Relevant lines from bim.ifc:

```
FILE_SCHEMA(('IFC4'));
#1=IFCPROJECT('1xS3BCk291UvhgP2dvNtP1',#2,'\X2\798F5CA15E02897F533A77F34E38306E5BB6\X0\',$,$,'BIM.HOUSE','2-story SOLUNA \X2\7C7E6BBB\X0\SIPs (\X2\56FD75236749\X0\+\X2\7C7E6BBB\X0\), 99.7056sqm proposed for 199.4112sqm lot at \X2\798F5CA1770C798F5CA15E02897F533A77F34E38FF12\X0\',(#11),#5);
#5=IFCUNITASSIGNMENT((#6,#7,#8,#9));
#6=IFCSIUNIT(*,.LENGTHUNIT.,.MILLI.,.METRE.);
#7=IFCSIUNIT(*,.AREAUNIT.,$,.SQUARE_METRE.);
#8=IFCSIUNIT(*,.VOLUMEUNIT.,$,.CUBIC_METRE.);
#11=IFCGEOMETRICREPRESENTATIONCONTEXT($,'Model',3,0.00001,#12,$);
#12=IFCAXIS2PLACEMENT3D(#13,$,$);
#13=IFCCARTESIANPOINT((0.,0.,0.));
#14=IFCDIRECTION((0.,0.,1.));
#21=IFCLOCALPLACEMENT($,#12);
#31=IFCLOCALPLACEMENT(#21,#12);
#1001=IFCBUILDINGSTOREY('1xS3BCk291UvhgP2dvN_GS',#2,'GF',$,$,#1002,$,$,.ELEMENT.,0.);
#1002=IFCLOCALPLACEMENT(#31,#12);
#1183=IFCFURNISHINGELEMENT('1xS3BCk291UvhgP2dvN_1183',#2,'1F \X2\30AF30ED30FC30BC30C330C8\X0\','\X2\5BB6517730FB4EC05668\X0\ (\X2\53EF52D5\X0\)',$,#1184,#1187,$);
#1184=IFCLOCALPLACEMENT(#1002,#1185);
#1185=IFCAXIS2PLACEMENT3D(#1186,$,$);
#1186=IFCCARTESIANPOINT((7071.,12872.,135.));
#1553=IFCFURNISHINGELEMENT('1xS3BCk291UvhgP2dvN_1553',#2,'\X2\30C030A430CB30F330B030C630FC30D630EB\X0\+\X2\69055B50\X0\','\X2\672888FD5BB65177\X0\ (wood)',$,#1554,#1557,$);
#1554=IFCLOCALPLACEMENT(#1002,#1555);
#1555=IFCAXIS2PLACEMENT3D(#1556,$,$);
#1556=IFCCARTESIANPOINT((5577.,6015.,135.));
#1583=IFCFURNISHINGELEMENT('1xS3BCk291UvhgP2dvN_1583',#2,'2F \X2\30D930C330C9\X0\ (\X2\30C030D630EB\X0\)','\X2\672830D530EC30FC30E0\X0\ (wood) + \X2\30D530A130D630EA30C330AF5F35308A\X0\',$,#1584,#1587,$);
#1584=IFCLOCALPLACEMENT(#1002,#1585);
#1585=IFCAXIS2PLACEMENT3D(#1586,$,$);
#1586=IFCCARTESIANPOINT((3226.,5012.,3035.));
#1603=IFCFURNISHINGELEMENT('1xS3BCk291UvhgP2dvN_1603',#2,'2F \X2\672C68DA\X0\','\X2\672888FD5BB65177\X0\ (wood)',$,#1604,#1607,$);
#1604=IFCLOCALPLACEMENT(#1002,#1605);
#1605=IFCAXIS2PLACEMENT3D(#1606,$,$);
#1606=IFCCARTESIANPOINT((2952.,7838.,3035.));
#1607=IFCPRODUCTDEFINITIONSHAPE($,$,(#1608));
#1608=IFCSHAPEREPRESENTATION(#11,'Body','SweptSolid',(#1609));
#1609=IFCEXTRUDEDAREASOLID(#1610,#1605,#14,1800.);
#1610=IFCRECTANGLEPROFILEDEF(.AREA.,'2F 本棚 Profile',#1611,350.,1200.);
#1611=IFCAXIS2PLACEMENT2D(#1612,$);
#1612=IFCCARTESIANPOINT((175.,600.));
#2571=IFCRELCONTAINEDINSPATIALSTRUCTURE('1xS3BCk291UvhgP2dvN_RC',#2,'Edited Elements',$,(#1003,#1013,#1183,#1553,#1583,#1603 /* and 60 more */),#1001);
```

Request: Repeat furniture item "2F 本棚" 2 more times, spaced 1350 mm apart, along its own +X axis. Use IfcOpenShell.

```python
import ifcopenshell
import ifcopenshell.api.geometry
import ifcopenshell.api.root
import ifcopenshell.util.element
import ifcopenshell.util.placement
import ifcopenshell.util.unit

model = ifcopenshell.open("bim.ifc")
unit_scale = ifcopenshell.util.unit.calculate_unit_scale(model)


def reuse_history(source, copy):
    """copy_class also copies each property set's owner history, people and application; keep the originals."""
    for rel in copy.IsDefinedBy:
        if rel.is_a("IfcRelDefinesByProperties") and (history := rel.RelatingPropertyDefinition.OwnerHistory):
            rel.RelatingPropertyDefinition.OwnerHistory = source.OwnerHistory
            ifcopenshell.util.element.remove_deep2(model, history)


source = model.by_id(1603)
base = ifcopenshell.util.placement.get_local_placement(source.ObjectPlacement)
step = base[:3, 0] * 1.35 / unit_scale

for i in range(1, 3):
    copy = ifcopenshell.api.root.copy_class(model, product=source)
    copy.Representation = ifcopenshell.util.element.copy_deep(
        model, source.Representation, exclude=["IfcGeometricRepresentationContext", "IfcRepresentationMap"]
    )
    reuse_history(source, copy)
    matrix = base.copy()
    matrix[:3, 3] += i * step
    print("added at", matrix[:3, 3].round(3) + 0.0)
    ifcopenshell.api.geometry.edit_object_placement(model, product=copy, matrix=matrix, is_si=False)

model.write("bim_rev.ifc")
```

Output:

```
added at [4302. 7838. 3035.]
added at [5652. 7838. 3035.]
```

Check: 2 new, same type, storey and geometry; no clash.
